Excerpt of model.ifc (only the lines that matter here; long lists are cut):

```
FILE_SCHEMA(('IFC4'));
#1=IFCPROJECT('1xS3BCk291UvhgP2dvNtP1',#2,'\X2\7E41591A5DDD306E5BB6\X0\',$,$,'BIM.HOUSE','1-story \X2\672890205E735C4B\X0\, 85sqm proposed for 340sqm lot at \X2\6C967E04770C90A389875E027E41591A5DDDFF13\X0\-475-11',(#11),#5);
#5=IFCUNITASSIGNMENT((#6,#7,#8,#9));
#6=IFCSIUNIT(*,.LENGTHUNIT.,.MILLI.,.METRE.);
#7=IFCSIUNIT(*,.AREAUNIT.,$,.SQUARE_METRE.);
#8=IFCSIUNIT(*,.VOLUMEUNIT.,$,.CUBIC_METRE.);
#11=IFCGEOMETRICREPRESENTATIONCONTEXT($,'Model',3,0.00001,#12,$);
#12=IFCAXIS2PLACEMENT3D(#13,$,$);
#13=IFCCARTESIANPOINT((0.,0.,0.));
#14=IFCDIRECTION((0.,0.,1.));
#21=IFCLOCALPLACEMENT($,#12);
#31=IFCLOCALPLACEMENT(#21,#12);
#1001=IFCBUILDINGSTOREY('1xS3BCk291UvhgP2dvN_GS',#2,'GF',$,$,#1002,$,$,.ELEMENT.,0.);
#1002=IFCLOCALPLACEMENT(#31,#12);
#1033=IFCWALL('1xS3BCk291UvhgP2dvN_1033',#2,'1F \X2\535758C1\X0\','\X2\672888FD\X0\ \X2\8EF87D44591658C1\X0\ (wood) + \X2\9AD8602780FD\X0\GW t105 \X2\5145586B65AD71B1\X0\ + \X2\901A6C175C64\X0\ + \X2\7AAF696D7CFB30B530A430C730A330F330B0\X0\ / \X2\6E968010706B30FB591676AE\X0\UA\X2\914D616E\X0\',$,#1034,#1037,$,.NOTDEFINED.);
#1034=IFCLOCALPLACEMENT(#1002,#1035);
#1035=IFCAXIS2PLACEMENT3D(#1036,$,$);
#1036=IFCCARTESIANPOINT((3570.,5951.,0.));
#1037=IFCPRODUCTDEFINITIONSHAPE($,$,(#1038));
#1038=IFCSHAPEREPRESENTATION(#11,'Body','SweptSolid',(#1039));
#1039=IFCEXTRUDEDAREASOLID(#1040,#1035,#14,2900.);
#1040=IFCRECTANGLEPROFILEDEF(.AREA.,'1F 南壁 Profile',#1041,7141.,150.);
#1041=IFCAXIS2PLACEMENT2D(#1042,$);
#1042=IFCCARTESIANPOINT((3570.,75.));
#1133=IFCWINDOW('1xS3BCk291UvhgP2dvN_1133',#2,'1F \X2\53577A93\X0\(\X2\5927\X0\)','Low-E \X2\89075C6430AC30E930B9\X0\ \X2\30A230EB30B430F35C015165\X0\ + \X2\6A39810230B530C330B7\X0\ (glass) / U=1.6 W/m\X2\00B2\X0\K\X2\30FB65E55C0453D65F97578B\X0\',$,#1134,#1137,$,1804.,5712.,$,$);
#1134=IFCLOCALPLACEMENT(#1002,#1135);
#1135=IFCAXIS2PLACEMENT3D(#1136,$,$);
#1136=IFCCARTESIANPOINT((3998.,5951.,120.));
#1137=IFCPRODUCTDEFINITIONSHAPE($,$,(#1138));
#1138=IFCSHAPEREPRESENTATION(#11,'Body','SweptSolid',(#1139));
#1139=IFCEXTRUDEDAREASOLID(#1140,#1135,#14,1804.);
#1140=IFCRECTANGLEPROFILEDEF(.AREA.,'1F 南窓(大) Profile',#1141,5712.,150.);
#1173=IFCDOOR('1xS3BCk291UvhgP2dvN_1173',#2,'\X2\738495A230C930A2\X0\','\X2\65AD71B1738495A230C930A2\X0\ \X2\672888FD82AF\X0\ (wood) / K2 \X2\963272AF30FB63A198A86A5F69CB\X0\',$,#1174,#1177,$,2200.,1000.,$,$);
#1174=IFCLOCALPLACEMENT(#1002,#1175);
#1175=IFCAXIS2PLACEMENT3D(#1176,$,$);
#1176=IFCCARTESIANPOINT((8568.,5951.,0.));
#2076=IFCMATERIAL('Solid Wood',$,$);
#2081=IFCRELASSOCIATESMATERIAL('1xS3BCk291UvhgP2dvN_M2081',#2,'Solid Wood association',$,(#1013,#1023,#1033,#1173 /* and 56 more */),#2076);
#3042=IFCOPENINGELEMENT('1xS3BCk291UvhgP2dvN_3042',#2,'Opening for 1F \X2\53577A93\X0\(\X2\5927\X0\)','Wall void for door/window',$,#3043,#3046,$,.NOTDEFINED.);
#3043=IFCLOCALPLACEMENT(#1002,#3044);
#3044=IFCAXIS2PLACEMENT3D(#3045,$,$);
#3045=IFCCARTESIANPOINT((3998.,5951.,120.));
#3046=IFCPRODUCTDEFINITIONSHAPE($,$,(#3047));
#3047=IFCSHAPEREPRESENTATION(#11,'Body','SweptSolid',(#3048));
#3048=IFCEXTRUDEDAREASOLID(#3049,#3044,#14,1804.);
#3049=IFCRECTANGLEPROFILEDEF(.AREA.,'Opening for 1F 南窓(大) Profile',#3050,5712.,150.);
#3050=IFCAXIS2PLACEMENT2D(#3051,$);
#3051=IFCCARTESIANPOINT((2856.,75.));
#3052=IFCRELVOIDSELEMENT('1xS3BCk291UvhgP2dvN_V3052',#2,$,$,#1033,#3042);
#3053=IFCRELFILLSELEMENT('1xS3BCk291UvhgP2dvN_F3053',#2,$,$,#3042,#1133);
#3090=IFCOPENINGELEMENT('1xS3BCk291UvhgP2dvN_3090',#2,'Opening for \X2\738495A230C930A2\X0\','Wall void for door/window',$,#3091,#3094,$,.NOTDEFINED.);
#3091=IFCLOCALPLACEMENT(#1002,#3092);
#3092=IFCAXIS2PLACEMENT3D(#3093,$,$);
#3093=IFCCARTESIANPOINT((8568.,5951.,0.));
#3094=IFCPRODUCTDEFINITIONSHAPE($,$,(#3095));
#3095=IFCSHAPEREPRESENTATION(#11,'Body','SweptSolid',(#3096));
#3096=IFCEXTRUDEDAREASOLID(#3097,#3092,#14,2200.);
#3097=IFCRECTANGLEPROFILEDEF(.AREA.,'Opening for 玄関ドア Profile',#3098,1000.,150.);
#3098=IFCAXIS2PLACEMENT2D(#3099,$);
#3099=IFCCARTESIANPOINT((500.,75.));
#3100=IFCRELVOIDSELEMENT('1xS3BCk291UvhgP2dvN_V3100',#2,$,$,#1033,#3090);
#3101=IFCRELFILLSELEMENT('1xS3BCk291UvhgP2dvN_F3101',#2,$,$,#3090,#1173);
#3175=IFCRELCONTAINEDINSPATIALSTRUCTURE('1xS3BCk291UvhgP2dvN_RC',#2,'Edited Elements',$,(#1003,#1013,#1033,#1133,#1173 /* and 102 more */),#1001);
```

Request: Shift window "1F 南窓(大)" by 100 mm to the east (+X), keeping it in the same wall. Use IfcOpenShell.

```python
import ifcopenshell
import ifcopenshell.api.geometry
import ifcopenshell.util.placement

model = ifcopenshell.open("model.ifc")

window = model.by_guid("1xS3BCk291UvhgP2dvN_1133")
opening = window.FillsVoids[0].RelatingOpeningElement
wall = opening.VoidsElements[0].RelatingBuildingElement

wall_matrix = ifcopenshell.util.placement.get_local_placement(wall.ObjectPlacement)
shift = wall_matrix[:3, 0] * 100.0
before = ifcopenshell.util.placement.get_local_placement(window.ObjectPlacement)[:3, 3].copy()

# The window is not placed relative to its opening, so move both.
for product in (opening, window):
    matrix = ifcopenshell.util.placement.get_local_placement(product.ObjectPlacement)
    matrix[:3, 3] += shift
    ifcopenshell.api.geometry.edit_object_placement(model, product=product, matrix=matrix, is_si=False)

after = ifcopenshell.util.placement.get_local_placement(window.ObjectPlacement)[:3, 3]
print("window moved by", (after - before).round(3) + 0.0)

model.write("model-out.ifc")
```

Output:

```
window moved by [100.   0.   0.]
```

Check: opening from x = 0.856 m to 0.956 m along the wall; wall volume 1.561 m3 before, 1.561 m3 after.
